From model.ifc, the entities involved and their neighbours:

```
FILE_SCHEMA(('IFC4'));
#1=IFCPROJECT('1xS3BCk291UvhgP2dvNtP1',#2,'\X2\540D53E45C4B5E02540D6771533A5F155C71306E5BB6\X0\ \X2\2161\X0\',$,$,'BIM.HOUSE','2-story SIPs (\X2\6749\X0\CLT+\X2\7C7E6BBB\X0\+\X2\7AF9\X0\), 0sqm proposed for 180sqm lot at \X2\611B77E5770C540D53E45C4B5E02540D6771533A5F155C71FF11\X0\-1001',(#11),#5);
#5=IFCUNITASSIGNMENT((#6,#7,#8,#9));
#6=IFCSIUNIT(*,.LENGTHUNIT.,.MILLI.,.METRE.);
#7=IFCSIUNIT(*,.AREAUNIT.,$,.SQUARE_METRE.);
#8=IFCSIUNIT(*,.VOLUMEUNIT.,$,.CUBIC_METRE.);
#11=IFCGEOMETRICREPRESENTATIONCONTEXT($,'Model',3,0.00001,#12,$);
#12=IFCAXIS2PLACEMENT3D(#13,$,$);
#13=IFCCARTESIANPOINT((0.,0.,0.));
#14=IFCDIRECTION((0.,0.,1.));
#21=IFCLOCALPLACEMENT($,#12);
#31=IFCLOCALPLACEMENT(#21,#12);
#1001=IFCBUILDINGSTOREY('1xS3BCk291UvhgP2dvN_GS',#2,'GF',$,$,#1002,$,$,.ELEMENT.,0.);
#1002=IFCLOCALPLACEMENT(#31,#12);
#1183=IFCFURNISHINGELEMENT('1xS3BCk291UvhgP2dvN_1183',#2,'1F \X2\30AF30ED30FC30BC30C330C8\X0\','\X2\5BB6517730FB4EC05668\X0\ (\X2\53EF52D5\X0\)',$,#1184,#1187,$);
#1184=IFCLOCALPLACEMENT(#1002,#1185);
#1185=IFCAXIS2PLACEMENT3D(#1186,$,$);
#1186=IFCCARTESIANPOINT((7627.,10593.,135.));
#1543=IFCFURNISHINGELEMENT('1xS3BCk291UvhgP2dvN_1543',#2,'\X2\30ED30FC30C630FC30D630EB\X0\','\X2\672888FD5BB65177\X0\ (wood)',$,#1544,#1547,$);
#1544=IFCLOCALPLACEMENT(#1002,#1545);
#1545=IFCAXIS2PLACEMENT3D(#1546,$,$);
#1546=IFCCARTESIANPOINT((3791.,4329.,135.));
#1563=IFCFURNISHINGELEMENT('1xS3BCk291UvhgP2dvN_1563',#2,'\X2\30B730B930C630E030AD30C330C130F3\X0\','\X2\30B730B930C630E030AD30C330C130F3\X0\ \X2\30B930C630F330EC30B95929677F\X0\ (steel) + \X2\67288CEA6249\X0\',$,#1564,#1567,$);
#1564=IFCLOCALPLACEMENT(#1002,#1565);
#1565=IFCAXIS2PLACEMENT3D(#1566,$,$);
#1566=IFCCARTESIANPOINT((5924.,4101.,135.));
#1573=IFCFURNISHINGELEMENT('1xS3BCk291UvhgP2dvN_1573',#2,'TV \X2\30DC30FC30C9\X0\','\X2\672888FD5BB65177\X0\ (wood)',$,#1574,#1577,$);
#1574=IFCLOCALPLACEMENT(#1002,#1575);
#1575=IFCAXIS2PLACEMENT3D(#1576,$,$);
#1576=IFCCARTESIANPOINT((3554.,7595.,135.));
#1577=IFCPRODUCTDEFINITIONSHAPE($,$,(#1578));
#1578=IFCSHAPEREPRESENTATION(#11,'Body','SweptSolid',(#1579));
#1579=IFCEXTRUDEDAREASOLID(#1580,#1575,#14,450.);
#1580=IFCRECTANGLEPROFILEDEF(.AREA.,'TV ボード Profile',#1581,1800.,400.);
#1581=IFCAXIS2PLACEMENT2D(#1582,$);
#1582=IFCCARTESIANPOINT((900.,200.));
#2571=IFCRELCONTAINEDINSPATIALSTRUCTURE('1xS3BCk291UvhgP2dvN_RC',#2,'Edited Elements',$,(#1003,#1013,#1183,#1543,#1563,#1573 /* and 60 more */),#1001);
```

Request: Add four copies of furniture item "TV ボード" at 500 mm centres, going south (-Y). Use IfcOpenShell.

```python
import numpy as np
import ifcopenshell
import ifcopenshell.api.geometry
import ifcopenshell.api.root
import ifcopenshell.util.element
import ifcopenshell.util.placement

model = ifcopenshell.open("model.ifc")


def reuse_history(source, copy):
    """copy_class also copies each property set's owner history, people and application; keep the originals."""
    for rel in copy.IsDefinedBy:
        if rel.is_a("IfcRelDefinesByProperties") and (history := rel.RelatingPropertyDefinition.OwnerHistory):
            rel.RelatingPropertyDefinition.OwnerHistory = source.OwnerHistory
            ifcopenshell.util.element.remove_deep2(model, history)


source = model.by_guid("1xS3BCk291UvhgP2dvN_1573")
base = ifcopenshell.util.placement.get_local_placement(source.ObjectPlacement)
step = np.array([0.0, -1.0, 0.0]) * 500.0

for i in range(1, 5):
    copy = ifcopenshell.api.root.copy_class(model, product=source)
    copy.Representation = ifcopenshell.util.element.copy_deep(
        model, source.Representation, exclude=["IfcGeometricRepresentationContext", "IfcRepresentationMap"]
    )
    reuse_history(source, copy)
    matrix = base.copy()
    matrix[:3, 3] += i * step
    print("added at", matrix[:3, 3].round(3) + 0.0)
    ifcopenshell.api.geometry.edit_object_placement(model, product=copy, matrix=matrix, is_si=False)

model.write("model_v2.ifc")
```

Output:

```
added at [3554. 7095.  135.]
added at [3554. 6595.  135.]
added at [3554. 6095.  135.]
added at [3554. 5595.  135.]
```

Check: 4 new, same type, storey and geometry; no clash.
